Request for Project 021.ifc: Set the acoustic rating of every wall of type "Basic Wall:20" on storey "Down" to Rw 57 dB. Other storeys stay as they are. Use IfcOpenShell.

First a look at what the model holds.

```python
import ifcopenshell
import ifcopenshell.util.element

model = ifcopenshell.open("Project 021.ifc")
print(model.schema)
storey = next(s for s in model.by_type("IfcBuildingStorey") if s.Name == "Down")
walls = [e for e in ifcopenshell.util.element.get_decomposition(storey) if e.is_a("IfcWall")]
seen = {}
for e in walls:
    element_type = ifcopenshell.util.element.get_type(e)
    key = (element_type.Name if element_type != e and element_type else None, ifcopenshell.util.element.get_pset(e, "Pset_WallCommon", "AcousticRating"))
    seen[key] = seen.get(key, 0) + 1
for (name, value), count in sorted(seen.items(), key=str):
    print(count, "x", name, "|", value)
```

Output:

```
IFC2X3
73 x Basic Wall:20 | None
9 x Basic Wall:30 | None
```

```python
import ifcopenshell
import ifcopenshell.api.pset
import ifcopenshell.util.element

model = ifcopenshell.open("Project 021.ifc")

storey = next(s for s in model.by_type("IfcBuildingStorey") if s.Name == "Down")
walls = [e for e in ifcopenshell.util.element.get_decomposition(storey) if e.is_a("IfcWall")]

count = 0
for e in walls:
    element_type = ifcopenshell.util.element.get_type(e)
    if element_type in (None, e) or element_type.Name != "Basic Wall:20":
        continue
    # add_pset returns the element's existing set when there is one.
    pset = ifcopenshell.api.pset.add_pset(model, product=e, name="Pset_WallCommon")
    ifcopenshell.api.pset.edit_pset(model, pset=pset, properties={"AcousticRating": "Rw 57 dB"})
    count += 1

print(count, "walls updated")

model.write("Project 021_edited.ifc")
```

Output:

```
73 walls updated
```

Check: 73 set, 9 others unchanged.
